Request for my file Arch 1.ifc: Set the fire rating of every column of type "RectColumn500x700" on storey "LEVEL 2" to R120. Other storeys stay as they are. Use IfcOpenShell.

First a look at what the model holds.

```python
import ifcopenshell
import ifcopenshell.util.element

model = ifcopenshell.open("my file Arch 1.ifc")
print(model.schema)
storey = next(s for s in model.by_type("IfcBuildingStorey") if s.Name == "LEVEL 2")
columns = [e for e in ifcopenshell.util.element.get_decomposition(storey) if e.is_a("IfcColumn")]
seen = {}
for e in columns:
    element_type = ifcopenshell.util.element.get_type(e)
    key = (element_type.Name if element_type != e and element_type else None, ifcopenshell.util.element.get_pset(e, "Pset_ColumnCommon", "FireRating"))
    seen[key] = seen.get(key, 0) + 1
for (name, value), count in sorted(seen.items(), key=str):
    print(count, "x", name, "|", value)
```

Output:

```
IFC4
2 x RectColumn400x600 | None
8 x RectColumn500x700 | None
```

```python
import ifcopenshell
import ifcopenshell.api.pset
import ifcopenshell.util.element

model = ifcopenshell.open("my file Arch 1.ifc")

storey = next(s for s in model.by_type("IfcBuildingStorey") if s.Name == "LEVEL 2")
columns = [e for e in ifcopenshell.util.element.get_decomposition(storey) if e.is_a("IfcColumn")]

count = 0
for e in columns:
    element_type = ifcopenshell.util.element.get_type(e)
    if element_type in (None, e) or element_type.Name != "RectColumn500x700":
        continue
    # add_pset returns the element's existing set when there is one.
    pset = ifcopenshell.api.pset.add_pset(model, product=e, name="Pset_ColumnCommon")
    ifcopenshell.api.pset.edit_pset(model, pset=pset, properties={"FireRating": "R120"})
    count += 1

print(count, "columns updated")

model.write("my file Arch 1_updated.ifc")
```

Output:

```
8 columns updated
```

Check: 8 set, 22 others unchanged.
